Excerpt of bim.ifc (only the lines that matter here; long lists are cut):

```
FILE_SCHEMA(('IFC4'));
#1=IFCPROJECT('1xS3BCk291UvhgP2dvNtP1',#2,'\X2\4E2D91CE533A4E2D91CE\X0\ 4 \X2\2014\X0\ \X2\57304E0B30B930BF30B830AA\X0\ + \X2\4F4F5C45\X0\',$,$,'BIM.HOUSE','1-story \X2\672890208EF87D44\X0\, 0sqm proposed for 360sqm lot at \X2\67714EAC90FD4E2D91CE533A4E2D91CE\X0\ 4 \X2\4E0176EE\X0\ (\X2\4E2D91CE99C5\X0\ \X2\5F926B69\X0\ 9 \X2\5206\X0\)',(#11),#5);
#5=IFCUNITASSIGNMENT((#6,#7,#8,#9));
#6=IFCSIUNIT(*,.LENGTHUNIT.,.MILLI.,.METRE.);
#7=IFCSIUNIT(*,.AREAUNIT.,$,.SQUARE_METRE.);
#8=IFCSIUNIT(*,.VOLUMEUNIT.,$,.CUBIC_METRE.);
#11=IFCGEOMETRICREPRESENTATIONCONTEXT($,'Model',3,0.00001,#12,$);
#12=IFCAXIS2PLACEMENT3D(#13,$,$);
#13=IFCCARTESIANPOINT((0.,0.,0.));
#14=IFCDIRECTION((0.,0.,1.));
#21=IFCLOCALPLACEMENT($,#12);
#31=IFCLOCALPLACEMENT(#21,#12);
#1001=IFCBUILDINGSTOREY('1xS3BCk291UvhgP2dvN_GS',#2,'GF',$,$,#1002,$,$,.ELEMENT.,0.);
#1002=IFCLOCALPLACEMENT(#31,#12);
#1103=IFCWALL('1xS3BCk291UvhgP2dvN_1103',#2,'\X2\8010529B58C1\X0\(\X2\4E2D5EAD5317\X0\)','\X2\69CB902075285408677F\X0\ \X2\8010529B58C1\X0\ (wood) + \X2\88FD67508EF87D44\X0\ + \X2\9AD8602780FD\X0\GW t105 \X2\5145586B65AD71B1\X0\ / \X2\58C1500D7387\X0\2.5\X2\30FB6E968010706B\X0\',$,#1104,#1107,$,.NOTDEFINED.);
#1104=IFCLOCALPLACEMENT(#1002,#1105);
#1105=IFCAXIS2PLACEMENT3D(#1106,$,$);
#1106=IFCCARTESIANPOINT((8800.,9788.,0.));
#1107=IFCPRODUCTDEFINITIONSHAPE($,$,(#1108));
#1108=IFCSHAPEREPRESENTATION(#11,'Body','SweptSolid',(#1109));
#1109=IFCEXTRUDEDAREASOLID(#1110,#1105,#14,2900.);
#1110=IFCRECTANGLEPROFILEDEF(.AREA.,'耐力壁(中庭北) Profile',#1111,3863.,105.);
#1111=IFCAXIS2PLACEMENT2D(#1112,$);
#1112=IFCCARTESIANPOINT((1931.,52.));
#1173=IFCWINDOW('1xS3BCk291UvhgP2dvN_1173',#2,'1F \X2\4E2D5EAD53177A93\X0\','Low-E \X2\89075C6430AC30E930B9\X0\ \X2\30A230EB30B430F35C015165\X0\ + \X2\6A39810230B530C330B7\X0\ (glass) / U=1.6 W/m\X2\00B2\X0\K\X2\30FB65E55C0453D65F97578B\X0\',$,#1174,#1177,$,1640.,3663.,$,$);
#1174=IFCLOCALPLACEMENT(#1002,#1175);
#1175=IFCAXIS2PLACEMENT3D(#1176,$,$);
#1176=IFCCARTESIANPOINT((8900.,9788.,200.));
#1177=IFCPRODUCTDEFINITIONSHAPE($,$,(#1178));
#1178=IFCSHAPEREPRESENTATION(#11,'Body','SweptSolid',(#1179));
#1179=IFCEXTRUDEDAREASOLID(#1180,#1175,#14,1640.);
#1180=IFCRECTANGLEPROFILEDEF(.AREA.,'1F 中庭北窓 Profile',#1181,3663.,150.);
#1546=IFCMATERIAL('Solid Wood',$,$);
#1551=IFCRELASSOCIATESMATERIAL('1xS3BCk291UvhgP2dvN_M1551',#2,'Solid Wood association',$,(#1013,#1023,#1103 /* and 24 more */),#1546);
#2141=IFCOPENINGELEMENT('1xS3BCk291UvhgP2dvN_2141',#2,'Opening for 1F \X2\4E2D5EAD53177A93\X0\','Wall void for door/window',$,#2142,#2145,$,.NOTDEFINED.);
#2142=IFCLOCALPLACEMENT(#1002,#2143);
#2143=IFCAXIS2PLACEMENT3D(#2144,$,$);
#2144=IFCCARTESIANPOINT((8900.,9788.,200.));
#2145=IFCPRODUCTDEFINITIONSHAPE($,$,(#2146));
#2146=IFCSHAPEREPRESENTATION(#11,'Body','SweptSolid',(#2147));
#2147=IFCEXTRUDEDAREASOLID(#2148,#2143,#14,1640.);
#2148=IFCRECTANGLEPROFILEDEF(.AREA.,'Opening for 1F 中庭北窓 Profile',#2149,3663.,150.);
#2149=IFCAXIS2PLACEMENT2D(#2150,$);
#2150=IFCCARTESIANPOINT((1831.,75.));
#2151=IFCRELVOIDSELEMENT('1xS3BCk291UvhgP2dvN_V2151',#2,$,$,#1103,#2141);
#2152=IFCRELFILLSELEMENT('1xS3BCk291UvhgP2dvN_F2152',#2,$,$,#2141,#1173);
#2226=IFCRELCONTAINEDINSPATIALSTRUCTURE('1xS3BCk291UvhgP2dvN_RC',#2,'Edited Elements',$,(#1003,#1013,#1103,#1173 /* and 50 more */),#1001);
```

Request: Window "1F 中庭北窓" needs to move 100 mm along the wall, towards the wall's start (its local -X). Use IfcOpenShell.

```python
import ifcopenshell
import ifcopenshell.api.geometry
import ifcopenshell.util.placement
import ifcopenshell.util.unit

model = ifcopenshell.open("bim.ifc")
unit_scale = ifcopenshell.util.unit.calculate_unit_scale(model)

window = model.by_guid("1xS3BCk291UvhgP2dvN_1173")
opening = window.FillsVoids[0].RelatingOpeningElement
wall = opening.VoidsElements[0].RelatingBuildingElement

wall_matrix = ifcopenshell.util.placement.get_local_placement(wall.ObjectPlacement)
shift = wall_matrix[:3, 0] * -0.1 / unit_scale
before = ifcopenshell.util.placement.get_local_placement(window.ObjectPlacement)[:3, 3].copy()

# The window is not placed relative to its opening, so move both.
for product in (opening, window):
    matrix = ifcopenshell.util.placement.get_local_placement(product.ObjectPlacement)
    matrix[:3, 3] += shift
    ifcopenshell.api.geometry.edit_object_placement(model, product=product, matrix=matrix, is_si=False)

after = ifcopenshell.util.placement.get_local_placement(window.ObjectPlacement)[:3, 3]
print("window moved by", (after - before).round(3) + 0.0)

model.write("bim_rev.ifc")
```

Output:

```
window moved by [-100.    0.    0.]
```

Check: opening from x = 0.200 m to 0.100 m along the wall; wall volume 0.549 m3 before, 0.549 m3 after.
